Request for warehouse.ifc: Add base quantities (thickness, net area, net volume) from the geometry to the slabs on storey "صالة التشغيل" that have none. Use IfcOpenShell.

First a look at what the model holds.

```python
import ifcopenshell
import ifcopenshell.util.element
import ifcopenshell.util.unit

model = ifcopenshell.open("warehouse.ifc")
print(model.schema)
for unit_type in ("LENGTHUNIT", "AREAUNIT", "VOLUMEUNIT"):
    print(unit_type, ifcopenshell.util.unit.calculate_unit_scale(model, unit_type))
storey = next(s for s in model.by_type("IfcBuildingStorey") if s.Name == "صالة التشغيل")
slabs = [e for e in ifcopenshell.util.element.get_decomposition(storey) if e.is_a("IfcSlab")]
for e in sorted(slabs, key=lambda e: e.id()):
    print(e.id(), e.is_a(), e.Name, list(ifcopenshell.util.element.get_psets(e, qtos_only=True)), sep=" | ")
```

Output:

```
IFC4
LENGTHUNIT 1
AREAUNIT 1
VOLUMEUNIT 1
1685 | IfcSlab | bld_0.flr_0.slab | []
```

```python
import ifcopenshell
import ifcopenshell.api.pset
import ifcopenshell.geom
import ifcopenshell.util.element
import ifcopenshell.util.shape
import ifcopenshell.util.unit

model = ifcopenshell.open("warehouse.ifc")
unit_scale = ifcopenshell.util.unit.calculate_unit_scale(model)
area_scale = ifcopenshell.util.unit.calculate_unit_scale(model, "AREAUNIT")
volume_scale = ifcopenshell.util.unit.calculate_unit_scale(model, "VOLUMEUNIT")
settings = ifcopenshell.geom.settings()

storey = next(s for s in model.by_type("IfcBuildingStorey") if s.Name == "صالة التشغيل")
slabs = [e for e in ifcopenshell.util.element.get_decomposition(storey) if e.is_a("IfcSlab")]

for e in sorted(slabs, key=lambda e: e.id()):
    if ifcopenshell.util.element.get_psets(e, qtos_only=True, should_inherit=False):
        continue
    # Geometry comes back in metres, in the element's own axes.
    shape = ifcopenshell.geom.create_shape(settings, e)
    values = {
        "Width": ifcopenshell.util.shape.get_z(shape.geometry) / unit_scale,
        "NetArea": ifcopenshell.util.shape.get_footprint_area(shape.geometry) / area_scale,
        "NetVolume": ifcopenshell.util.shape.get_volume(shape.geometry) / volume_scale,
    }
    qto = ifcopenshell.api.pset.add_qto(model, product=e, name="Qto_SlabBaseQuantities")
    ifcopenshell.api.pset.edit_qto(model, qto=qto, properties=values)
    print(e.id(), {k: round(v, 3) for k, v in values.items()})

model.write("warehouse_v2.ifc")
```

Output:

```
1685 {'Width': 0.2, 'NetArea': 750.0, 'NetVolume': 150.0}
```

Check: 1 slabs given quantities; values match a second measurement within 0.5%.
